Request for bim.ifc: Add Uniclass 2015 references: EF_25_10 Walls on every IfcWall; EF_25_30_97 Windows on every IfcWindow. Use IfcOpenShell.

First a look at what the model holds.

```python
import ifcopenshell

model = ifcopenshell.open("bim.ifc")
print(model.schema)
print("classifications:", [c.Name for c in model.by_type("IfcClassification")])
for ifc_class in ("IfcDoor", "IfcRoof", "IfcStair", "IfcWall", "IfcWindow"):
    print(ifc_class, len(model.by_type(ifc_class)))
```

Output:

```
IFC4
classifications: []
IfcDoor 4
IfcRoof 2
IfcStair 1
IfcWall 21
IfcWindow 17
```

```python
import ifcopenshell
import ifcopenshell.api.classification

model = ifcopenshell.open("bim.ifc")

system = ifcopenshell.api.classification.add_classification(model, classification="Uniclass 2015")

codes = {
    "IfcWall": ("EF_25_10", "Walls"),
    "IfcWindow": ("EF_25_30_97", "Windows"),
}
for ifc_class, (code, name) in codes.items():
    products = model.by_type(ifc_class)
    ifcopenshell.api.classification.add_reference(
        model, products=products, classification=system, identification=code, name=name
    )
    print(code, len(products))

model.write("bim-out.ifc")
```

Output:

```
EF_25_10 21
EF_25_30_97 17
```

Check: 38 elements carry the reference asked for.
